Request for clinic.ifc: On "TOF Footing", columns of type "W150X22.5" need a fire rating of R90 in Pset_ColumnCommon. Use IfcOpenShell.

First a look at what the model holds.

```python
import ifcopenshell
import ifcopenshell.util.element

model = ifcopenshell.open("clinic.ifc")
print(model.schema)
storey = next(s for s in model.by_type("IfcBuildingStorey") if s.Name == "TOF Footing")
columns = [e for e in ifcopenshell.util.element.get_decomposition(storey) if e.is_a("IfcColumn")]
seen = {}
for e in columns:
    element_type = ifcopenshell.util.element.get_type(e)
    key = (element_type.Name if element_type != e and element_type else None, ifcopenshell.util.element.get_pset(e, "Pset_ColumnCommon", "FireRating"))
    seen[key] = seen.get(key, 0) + 1
for (name, value), count in sorted(seen.items(), key=str):
    print(count, "x", name, "|", value)
```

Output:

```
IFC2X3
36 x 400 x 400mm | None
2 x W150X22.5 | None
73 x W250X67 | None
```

```python
import ifcopenshell
import ifcopenshell.api.pset
import ifcopenshell.util.element

model = ifcopenshell.open("clinic.ifc")

storey = next(s for s in model.by_type("IfcBuildingStorey") if s.Name == "TOF Footing")
columns = [e for e in ifcopenshell.util.element.get_decomposition(storey) if e.is_a("IfcColumn")]

count = 0
for e in columns:
    element_type = ifcopenshell.util.element.get_type(e)
    if element_type in (None, e) or element_type.Name != "W150X22.5":
        continue
    # add_pset returns the element's existing set when there is one.
    pset = ifcopenshell.api.pset.add_pset(model, product=e, name="Pset_ColumnCommon")
    ifcopenshell.api.pset.edit_pset(model, pset=pset, properties={"FireRating": "R90"})
    count += 1

print(count, "columns updated")

model.write("clinic_rev.ifc")
```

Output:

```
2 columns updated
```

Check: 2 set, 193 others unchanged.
